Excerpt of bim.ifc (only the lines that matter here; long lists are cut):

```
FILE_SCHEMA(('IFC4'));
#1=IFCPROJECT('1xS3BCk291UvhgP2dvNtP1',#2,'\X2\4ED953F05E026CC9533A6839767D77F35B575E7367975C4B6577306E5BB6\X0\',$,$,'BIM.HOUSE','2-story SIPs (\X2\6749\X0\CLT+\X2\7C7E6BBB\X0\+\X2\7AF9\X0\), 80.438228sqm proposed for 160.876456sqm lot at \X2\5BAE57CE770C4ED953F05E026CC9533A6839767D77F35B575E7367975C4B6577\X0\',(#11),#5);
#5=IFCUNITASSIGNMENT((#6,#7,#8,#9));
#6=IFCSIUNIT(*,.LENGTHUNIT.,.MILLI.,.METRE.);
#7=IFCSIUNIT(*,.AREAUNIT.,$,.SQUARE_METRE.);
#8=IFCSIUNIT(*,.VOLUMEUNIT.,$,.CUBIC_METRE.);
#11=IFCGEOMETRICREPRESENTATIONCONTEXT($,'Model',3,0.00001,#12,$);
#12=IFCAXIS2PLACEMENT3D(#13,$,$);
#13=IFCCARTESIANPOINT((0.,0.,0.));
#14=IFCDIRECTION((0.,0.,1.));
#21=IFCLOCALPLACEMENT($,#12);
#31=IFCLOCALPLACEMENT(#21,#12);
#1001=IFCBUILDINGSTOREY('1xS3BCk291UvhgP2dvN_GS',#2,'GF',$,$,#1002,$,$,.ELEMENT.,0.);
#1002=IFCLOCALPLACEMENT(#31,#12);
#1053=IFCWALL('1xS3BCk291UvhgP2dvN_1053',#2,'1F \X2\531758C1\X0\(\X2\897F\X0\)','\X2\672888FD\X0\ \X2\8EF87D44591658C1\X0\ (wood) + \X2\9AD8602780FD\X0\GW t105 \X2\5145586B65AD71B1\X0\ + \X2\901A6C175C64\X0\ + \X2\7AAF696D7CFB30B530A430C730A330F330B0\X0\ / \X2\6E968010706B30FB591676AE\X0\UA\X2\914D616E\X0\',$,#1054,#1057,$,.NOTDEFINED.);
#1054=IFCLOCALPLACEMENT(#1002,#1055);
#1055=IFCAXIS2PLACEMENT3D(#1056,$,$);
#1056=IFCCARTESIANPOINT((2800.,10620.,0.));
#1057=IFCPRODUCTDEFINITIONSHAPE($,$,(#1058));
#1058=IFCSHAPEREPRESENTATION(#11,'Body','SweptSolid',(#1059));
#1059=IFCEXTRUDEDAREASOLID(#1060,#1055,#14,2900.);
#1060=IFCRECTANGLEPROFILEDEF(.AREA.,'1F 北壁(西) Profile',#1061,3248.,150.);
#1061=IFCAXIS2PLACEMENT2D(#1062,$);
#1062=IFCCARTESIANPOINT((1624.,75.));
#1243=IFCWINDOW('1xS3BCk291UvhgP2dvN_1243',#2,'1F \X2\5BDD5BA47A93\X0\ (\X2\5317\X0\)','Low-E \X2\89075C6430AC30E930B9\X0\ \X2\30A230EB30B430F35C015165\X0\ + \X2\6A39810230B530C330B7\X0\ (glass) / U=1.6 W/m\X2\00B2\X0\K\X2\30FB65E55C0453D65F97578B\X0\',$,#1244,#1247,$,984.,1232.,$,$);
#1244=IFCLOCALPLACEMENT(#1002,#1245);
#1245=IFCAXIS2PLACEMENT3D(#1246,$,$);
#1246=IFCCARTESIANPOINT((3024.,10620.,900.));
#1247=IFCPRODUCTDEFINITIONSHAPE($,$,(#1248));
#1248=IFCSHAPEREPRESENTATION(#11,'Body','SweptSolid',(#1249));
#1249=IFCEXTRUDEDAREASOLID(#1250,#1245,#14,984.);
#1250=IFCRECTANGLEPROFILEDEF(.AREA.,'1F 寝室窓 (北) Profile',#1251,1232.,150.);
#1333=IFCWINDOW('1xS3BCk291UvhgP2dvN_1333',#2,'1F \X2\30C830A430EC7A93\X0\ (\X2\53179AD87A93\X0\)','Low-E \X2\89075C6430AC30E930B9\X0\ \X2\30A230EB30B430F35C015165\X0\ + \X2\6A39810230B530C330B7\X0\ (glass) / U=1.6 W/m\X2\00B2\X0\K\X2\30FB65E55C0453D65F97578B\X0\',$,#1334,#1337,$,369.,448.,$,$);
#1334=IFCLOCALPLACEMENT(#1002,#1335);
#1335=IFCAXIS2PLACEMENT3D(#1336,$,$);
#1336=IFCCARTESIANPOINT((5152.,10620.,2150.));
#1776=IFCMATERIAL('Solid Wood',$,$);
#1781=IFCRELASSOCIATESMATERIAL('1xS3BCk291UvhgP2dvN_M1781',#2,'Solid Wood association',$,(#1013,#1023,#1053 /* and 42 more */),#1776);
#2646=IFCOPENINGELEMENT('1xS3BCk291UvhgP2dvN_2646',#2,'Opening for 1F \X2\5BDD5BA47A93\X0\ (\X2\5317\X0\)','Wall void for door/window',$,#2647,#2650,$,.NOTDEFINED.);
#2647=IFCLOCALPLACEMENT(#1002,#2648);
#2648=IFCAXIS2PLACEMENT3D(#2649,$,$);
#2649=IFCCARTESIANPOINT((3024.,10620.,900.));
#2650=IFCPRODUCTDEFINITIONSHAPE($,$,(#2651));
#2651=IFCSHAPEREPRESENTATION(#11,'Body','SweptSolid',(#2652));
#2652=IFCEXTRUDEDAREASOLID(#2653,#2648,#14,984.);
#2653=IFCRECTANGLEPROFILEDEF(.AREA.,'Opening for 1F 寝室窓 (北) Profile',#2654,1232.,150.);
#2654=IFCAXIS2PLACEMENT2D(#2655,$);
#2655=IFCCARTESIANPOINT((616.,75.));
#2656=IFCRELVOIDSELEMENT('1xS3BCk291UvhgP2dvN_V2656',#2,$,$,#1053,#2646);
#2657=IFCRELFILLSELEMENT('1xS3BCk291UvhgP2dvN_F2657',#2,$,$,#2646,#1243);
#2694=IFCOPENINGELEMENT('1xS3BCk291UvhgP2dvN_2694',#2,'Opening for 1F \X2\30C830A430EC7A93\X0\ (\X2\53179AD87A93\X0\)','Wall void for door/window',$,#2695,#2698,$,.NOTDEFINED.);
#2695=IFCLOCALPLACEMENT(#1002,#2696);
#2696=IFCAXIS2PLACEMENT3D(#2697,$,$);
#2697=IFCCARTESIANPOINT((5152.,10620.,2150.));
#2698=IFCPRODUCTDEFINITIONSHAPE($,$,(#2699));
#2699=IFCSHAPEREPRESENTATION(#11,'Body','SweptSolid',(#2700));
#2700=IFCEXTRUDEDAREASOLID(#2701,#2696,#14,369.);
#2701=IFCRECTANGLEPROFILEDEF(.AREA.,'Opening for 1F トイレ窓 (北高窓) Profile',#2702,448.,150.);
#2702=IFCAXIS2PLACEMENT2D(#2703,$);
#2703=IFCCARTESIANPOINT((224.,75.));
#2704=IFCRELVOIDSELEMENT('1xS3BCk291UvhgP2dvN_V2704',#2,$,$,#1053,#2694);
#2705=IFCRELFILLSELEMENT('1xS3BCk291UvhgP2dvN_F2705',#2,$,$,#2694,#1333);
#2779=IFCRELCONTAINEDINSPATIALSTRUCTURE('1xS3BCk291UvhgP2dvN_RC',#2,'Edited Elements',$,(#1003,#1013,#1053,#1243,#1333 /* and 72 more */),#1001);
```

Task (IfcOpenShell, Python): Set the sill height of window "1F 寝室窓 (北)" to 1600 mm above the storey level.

```python
import numpy as np
import ifcopenshell
import ifcopenshell.api.geometry
import ifcopenshell.geom
import ifcopenshell.util.element
import ifcopenshell.util.placement
import ifcopenshell.util.shape
import ifcopenshell.util.unit

model = ifcopenshell.open("bim.ifc")
unit_scale = ifcopenshell.util.unit.calculate_unit_scale(model)

window = model.by_id(1243)
opening = window.FillsVoids[0].RelatingOpeningElement
storey = ifcopenshell.util.element.get_container(window, ifc_class="IfcBuildingStorey")
level = ifcopenshell.util.placement.get_local_placement(storey.ObjectPlacement)[2, 3]

# The opening's origin need not be at the sill, so measure its lowest point.
shape = ifcopenshell.geom.create_shape(ifcopenshell.geom.settings(), opening)
bottom = ifcopenshell.util.shape.get_shape_bottom_elevation(shape, shape.geometry) / unit_scale
dz = level + 1.6 / unit_scale - bottom

shift = np.array([0.0, 0.0, dz])
# The window is not placed relative to its opening, so move both.
for product in (opening, window):
    matrix = ifcopenshell.util.placement.get_local_placement(product.ObjectPlacement)
    matrix[:3, 3] += shift
    ifcopenshell.api.geometry.edit_object_placement(model, product=product, matrix=matrix, is_si=False)

print(f"moved by {dz * unit_scale:+.3f} m")

model.write("bim_updated.ifc")
```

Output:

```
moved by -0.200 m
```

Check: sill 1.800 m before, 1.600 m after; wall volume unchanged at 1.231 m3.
